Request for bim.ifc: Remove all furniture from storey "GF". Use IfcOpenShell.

First a look at what the model holds.

```python
import ifcopenshell
import ifcopenshell.util.element

model = ifcopenshell.open("bim.ifc")
print(model.schema)
storey = next(s for s in model.by_type("IfcBuildingStorey") if s.Name == "GF")
furniture = [e for e in ifcopenshell.util.element.get_decomposition(storey) if e.is_a("IfcFurnishingElement")]
seen = {}
for e in furniture:
    element_type = ifcopenshell.util.element.get_type(e)
    name = element_type.Name if element_type not in (None, e) else None
    seen[name] = seen.get(name, 0) + 1
for name, count in sorted(seen.items(), key=str):
    print(count, "x", name)
```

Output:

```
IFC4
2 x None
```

```python
import ifcopenshell
import ifcopenshell.api.root
import ifcopenshell.util.element

model = ifcopenshell.open("bim.ifc")

storey = next(s for s in model.by_type("IfcBuildingStorey") if s.Name == "GF")
furniture = [e for e in ifcopenshell.util.element.get_decomposition(storey) if e.is_a("IfcFurnishingElement")]

for e in furniture:
    ifcopenshell.api.root.remove_product(model, product=e)
print(len(furniture), "removed")

model.write("bim_updated.ifc")
```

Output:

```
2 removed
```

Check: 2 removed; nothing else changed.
